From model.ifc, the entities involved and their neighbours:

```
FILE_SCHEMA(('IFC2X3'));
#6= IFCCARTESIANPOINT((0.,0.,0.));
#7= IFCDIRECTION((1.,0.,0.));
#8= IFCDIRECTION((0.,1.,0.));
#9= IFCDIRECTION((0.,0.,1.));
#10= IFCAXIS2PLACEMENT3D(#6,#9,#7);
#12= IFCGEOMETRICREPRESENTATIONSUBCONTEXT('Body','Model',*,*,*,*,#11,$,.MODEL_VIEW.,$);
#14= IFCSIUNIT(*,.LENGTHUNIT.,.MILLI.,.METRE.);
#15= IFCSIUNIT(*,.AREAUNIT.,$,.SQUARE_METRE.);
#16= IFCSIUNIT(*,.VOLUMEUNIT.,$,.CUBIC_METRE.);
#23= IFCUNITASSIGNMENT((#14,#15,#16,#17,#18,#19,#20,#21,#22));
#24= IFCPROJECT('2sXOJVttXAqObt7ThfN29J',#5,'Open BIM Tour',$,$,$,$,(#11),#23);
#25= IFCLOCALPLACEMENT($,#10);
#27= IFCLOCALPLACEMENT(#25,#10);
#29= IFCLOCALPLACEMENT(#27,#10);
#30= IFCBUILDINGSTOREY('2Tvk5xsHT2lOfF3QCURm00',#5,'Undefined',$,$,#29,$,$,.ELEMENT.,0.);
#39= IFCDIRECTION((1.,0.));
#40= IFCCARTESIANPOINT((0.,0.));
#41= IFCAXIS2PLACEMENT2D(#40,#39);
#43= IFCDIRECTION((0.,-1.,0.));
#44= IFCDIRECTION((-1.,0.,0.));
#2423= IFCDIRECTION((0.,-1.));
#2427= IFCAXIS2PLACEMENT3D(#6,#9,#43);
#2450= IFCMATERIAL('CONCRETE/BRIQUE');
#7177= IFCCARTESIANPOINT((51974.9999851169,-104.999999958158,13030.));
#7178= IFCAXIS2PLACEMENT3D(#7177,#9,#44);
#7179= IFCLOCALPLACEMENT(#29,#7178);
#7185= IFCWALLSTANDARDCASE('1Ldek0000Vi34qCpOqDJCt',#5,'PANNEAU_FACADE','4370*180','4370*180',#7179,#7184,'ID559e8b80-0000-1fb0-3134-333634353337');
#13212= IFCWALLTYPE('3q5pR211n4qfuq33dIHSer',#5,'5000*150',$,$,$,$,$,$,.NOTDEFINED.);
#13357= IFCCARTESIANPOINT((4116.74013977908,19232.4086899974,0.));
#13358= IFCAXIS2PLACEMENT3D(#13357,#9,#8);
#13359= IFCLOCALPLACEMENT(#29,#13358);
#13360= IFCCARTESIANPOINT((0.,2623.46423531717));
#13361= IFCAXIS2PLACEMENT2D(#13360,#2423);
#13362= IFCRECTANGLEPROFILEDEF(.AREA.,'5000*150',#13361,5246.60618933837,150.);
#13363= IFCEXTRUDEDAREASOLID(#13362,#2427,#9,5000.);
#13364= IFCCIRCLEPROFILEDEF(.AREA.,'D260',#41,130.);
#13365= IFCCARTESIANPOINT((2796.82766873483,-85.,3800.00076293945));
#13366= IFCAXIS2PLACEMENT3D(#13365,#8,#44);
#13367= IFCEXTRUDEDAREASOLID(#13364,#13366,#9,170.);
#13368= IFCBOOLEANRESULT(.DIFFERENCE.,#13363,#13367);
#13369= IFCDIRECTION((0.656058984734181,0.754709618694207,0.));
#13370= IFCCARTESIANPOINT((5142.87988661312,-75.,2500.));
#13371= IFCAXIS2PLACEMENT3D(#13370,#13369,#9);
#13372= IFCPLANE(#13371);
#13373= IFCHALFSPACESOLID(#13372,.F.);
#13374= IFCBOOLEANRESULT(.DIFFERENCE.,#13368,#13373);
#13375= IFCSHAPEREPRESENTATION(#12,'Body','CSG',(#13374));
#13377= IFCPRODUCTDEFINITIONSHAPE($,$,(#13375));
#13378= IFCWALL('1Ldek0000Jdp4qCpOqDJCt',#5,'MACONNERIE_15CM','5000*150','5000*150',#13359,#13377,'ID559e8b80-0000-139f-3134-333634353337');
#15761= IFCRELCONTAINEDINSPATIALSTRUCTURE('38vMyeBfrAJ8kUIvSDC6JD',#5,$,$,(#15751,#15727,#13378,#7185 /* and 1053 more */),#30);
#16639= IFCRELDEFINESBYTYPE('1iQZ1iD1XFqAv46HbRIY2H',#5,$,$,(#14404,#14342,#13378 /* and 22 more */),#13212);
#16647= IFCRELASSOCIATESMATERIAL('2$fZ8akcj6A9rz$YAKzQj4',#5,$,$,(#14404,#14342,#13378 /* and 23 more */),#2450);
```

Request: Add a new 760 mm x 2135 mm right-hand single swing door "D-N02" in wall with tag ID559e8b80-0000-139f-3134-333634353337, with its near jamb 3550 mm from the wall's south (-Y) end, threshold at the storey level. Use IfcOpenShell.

```python
import numpy as np
import ifcopenshell
import ifcopenshell.api.feature
import ifcopenshell.api.geometry
import ifcopenshell.api.root
import ifcopenshell.api.spatial
import ifcopenshell.api.type
import ifcopenshell.geom
import ifcopenshell.util.element
import ifcopenshell.util.placement
import ifcopenshell.util.representation
import ifcopenshell.util.shape
import ifcopenshell.util.unit

model = ifcopenshell.open("model.ifc")
unit_scale = ifcopenshell.util.unit.calculate_unit_scale(model)
settings = ifcopenshell.geom.settings()


def volume(element):
    """Net volume in cubic metres, openings subtracted."""
    shape = ifcopenshell.geom.create_shape(settings, element)
    return ifcopenshell.util.shape.get_volume(shape.geometry)


wall = model.by_guid("1Ldek0000Jdp4qCpOqDJCt")
storey = ifcopenshell.util.element.get_container(wall, ifc_class="IfcBuildingStorey")
context = ifcopenshell.util.representation.get_context(model, "Model", "Body", "MODEL_VIEW")
before = volume(wall)

width, height, from_end, sill = 0.76, 2.135, 3.55, 0.0  # metres

# The wall runs along its own X axis, and the end named is its -X end.
wall_shape = ifcopenshell.geom.create_shape(settings, wall)
x, y, z = ifcopenshell.util.shape.get_vertices(wall_shape.geometry).T
start = x.min() + from_end
face, thickness = float(y.min()), float(y.max() - y.min())
wall_matrix = ifcopenshell.util.placement.get_local_placement(wall.ObjectPlacement)
level = ifcopenshell.util.placement.get_local_placement(storey.ObjectPlacement)[2, 3]


def in_wall(x, y):
    """Placement at x, y metres in the wall's axes, at sill height."""
    matrix = wall_matrix.copy()
    matrix[:, 3] = wall_matrix @ np.array([x / unit_scale, y / unit_scale, 0.0, 1.0])
    matrix[2, 3] = level + sill / unit_scale
    return matrix


# Opening: a box that overshoots both wall faces by 50 mm.
opening = ifcopenshell.api.root.create_entity(model, ifc_class="IfcOpeningElement")
box = ifcopenshell.api.geometry.add_wall_representation(
    model, context=context, length=width, height=height, thickness=thickness + 0.1
)
ifcopenshell.api.geometry.assign_representation(model, product=opening, representation=box)
ifcopenshell.api.geometry.edit_object_placement(model, product=opening, matrix=in_wall(start, face - 0.05), is_si=False)
ifcopenshell.api.feature.add_feature(model, feature=opening, element=wall)

door = ifcopenshell.api.root.create_entity(model, ifc_class="IfcDoor", name="D-N02")
door.OverallWidth, door.OverallHeight = width / unit_scale, height / unit_scale
body = ifcopenshell.api.geometry.add_door_representation(
    model,
    context=context,
    overall_width=door.OverallWidth,
    overall_height=door.OverallHeight,
    operation_type="SINGLE_SWING_RIGHT",
    lining_properties={"LiningDepth": thickness / unit_scale, "ThresholdDepth": thickness / unit_scale},
)
ifcopenshell.api.geometry.assign_representation(model, product=door, representation=body)
ifcopenshell.api.spatial.assign_container(model, products=[door], relating_structure=storey)
fills = ifcopenshell.api.feature.add_filling(model, opening=opening, element=door)
fills.OwnerHistory = door.OwnerHistory  # required in IFC2X3

# IFC2X3 keeps the operation on the door style.
style = ifcopenshell.api.root.create_entity(model, ifc_class="IfcDoorStyle", name="D-N02")
style.OperationType, style.ConstructionType = "SINGLE_SWING_RIGHT", "NOTDEFINED"
style.ParameterTakesPrecedence = style.Sizeable = False
ifcopenshell.api.type.assign_type(model, related_objects=[door], relating_type=style)

# The lining spans the wall, so the door starts at the wall face.
ifcopenshell.api.geometry.edit_object_placement(model, product=door, matrix=in_wall(start, face), is_si=False)

after = volume(wall)

print(f"wall volume {before:.3f} -> {after:.3f} m3")

model.write("model_updated.ifc")
```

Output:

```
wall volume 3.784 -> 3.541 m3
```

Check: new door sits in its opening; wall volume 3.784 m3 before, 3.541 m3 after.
